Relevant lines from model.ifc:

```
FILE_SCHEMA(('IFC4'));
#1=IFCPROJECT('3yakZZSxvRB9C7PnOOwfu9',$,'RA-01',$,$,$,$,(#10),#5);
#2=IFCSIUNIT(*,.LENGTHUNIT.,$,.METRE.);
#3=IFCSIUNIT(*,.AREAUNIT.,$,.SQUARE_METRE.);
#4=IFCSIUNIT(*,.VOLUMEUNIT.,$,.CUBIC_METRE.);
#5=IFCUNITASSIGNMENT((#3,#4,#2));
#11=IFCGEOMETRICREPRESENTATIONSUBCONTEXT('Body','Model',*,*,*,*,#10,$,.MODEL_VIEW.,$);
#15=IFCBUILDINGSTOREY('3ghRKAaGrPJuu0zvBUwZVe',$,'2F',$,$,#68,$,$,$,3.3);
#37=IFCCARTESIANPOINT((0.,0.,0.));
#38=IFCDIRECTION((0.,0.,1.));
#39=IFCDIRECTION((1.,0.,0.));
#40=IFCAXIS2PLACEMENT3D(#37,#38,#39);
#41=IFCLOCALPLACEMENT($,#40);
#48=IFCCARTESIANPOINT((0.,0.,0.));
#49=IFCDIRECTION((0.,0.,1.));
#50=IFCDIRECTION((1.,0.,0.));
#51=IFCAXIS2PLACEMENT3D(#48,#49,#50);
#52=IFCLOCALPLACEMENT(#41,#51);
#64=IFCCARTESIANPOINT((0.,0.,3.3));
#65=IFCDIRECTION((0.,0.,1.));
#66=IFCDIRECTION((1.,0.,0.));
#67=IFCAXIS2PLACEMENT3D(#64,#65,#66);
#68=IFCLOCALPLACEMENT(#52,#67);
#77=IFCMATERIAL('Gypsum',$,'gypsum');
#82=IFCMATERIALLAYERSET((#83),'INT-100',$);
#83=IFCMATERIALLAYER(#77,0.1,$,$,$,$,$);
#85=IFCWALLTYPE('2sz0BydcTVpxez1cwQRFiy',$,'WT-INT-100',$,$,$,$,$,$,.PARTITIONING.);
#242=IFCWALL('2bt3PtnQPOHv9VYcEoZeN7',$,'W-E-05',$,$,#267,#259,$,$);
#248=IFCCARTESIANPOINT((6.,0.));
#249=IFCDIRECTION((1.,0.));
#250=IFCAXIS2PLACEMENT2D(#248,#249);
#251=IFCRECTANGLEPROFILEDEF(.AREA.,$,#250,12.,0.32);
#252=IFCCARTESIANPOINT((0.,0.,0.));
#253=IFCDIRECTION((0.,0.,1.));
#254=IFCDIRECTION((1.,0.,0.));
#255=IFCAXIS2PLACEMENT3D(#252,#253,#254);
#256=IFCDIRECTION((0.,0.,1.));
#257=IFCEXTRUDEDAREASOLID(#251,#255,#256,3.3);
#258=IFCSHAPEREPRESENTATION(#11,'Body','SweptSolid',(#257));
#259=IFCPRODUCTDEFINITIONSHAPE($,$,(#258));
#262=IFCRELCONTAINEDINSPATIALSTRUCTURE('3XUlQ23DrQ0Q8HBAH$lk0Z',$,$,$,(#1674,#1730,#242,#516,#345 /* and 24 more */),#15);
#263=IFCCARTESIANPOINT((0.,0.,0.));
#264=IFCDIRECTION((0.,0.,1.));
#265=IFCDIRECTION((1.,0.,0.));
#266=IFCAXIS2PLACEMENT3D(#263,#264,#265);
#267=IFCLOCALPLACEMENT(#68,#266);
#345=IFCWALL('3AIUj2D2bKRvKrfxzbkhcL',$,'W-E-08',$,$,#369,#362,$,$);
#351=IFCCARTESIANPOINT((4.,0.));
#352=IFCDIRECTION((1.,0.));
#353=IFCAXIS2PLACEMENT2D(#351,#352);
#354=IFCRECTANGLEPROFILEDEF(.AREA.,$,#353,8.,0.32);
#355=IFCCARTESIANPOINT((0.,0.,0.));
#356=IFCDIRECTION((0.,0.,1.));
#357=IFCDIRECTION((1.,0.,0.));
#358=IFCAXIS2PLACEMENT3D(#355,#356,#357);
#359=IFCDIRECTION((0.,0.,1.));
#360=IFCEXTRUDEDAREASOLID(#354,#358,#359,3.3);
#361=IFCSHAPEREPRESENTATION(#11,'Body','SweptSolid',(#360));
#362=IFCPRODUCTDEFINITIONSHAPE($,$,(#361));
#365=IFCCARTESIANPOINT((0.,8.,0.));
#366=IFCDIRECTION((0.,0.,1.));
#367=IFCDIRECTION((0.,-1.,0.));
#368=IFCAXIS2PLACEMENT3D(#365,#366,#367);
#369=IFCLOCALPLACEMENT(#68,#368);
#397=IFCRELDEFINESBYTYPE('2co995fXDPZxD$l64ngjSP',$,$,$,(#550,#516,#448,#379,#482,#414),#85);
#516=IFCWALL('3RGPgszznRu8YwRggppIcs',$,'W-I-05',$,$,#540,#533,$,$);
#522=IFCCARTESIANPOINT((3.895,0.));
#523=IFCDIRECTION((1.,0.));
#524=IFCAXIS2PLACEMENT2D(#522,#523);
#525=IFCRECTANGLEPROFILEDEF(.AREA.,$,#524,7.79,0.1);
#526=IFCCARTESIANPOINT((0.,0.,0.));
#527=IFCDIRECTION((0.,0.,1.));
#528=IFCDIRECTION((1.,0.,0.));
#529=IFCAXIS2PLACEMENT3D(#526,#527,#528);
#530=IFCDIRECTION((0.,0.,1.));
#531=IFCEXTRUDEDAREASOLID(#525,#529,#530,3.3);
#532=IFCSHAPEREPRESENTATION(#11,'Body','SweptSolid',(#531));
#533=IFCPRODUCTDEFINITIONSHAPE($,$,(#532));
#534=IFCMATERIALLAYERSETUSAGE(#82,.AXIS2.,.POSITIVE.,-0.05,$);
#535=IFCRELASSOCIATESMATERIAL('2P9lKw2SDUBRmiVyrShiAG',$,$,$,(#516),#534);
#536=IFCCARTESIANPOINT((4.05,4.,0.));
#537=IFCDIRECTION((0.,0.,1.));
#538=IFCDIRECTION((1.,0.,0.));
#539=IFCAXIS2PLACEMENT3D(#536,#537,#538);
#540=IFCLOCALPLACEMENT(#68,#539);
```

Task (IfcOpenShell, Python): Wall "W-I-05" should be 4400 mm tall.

```python
import ifcopenshell
import ifcopenshell.geom
import ifcopenshell.util.representation
import ifcopenshell.util.shape
import ifcopenshell.util.unit

model = ifcopenshell.open("model.ifc")
unit_scale = ifcopenshell.util.unit.calculate_unit_scale(model)
settings = ifcopenshell.geom.settings()


def volume(element):
    """Net volume in cubic metres, openings subtracted."""
    shape = ifcopenshell.geom.create_shape(settings, element)
    return ifcopenshell.util.shape.get_volume(shape.geometry)


wall = model.by_guid("3RGPgszznRu8YwRggppIcs")
before = volume(wall)

body = ifcopenshell.util.representation.get_representation(wall, "Model", "Body")
solid = body.Items[0]
old_height = solid.Depth
solid.Depth = 4.4 / unit_scale
after = volume(wall)

print(f"height {old_height:g} -> {solid.Depth:g}, volume {before:.3f} -> {after:.3f} m3")

model.write("model_v2.ifc")
```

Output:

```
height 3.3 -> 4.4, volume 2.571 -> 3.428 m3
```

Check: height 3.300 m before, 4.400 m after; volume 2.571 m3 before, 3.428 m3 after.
